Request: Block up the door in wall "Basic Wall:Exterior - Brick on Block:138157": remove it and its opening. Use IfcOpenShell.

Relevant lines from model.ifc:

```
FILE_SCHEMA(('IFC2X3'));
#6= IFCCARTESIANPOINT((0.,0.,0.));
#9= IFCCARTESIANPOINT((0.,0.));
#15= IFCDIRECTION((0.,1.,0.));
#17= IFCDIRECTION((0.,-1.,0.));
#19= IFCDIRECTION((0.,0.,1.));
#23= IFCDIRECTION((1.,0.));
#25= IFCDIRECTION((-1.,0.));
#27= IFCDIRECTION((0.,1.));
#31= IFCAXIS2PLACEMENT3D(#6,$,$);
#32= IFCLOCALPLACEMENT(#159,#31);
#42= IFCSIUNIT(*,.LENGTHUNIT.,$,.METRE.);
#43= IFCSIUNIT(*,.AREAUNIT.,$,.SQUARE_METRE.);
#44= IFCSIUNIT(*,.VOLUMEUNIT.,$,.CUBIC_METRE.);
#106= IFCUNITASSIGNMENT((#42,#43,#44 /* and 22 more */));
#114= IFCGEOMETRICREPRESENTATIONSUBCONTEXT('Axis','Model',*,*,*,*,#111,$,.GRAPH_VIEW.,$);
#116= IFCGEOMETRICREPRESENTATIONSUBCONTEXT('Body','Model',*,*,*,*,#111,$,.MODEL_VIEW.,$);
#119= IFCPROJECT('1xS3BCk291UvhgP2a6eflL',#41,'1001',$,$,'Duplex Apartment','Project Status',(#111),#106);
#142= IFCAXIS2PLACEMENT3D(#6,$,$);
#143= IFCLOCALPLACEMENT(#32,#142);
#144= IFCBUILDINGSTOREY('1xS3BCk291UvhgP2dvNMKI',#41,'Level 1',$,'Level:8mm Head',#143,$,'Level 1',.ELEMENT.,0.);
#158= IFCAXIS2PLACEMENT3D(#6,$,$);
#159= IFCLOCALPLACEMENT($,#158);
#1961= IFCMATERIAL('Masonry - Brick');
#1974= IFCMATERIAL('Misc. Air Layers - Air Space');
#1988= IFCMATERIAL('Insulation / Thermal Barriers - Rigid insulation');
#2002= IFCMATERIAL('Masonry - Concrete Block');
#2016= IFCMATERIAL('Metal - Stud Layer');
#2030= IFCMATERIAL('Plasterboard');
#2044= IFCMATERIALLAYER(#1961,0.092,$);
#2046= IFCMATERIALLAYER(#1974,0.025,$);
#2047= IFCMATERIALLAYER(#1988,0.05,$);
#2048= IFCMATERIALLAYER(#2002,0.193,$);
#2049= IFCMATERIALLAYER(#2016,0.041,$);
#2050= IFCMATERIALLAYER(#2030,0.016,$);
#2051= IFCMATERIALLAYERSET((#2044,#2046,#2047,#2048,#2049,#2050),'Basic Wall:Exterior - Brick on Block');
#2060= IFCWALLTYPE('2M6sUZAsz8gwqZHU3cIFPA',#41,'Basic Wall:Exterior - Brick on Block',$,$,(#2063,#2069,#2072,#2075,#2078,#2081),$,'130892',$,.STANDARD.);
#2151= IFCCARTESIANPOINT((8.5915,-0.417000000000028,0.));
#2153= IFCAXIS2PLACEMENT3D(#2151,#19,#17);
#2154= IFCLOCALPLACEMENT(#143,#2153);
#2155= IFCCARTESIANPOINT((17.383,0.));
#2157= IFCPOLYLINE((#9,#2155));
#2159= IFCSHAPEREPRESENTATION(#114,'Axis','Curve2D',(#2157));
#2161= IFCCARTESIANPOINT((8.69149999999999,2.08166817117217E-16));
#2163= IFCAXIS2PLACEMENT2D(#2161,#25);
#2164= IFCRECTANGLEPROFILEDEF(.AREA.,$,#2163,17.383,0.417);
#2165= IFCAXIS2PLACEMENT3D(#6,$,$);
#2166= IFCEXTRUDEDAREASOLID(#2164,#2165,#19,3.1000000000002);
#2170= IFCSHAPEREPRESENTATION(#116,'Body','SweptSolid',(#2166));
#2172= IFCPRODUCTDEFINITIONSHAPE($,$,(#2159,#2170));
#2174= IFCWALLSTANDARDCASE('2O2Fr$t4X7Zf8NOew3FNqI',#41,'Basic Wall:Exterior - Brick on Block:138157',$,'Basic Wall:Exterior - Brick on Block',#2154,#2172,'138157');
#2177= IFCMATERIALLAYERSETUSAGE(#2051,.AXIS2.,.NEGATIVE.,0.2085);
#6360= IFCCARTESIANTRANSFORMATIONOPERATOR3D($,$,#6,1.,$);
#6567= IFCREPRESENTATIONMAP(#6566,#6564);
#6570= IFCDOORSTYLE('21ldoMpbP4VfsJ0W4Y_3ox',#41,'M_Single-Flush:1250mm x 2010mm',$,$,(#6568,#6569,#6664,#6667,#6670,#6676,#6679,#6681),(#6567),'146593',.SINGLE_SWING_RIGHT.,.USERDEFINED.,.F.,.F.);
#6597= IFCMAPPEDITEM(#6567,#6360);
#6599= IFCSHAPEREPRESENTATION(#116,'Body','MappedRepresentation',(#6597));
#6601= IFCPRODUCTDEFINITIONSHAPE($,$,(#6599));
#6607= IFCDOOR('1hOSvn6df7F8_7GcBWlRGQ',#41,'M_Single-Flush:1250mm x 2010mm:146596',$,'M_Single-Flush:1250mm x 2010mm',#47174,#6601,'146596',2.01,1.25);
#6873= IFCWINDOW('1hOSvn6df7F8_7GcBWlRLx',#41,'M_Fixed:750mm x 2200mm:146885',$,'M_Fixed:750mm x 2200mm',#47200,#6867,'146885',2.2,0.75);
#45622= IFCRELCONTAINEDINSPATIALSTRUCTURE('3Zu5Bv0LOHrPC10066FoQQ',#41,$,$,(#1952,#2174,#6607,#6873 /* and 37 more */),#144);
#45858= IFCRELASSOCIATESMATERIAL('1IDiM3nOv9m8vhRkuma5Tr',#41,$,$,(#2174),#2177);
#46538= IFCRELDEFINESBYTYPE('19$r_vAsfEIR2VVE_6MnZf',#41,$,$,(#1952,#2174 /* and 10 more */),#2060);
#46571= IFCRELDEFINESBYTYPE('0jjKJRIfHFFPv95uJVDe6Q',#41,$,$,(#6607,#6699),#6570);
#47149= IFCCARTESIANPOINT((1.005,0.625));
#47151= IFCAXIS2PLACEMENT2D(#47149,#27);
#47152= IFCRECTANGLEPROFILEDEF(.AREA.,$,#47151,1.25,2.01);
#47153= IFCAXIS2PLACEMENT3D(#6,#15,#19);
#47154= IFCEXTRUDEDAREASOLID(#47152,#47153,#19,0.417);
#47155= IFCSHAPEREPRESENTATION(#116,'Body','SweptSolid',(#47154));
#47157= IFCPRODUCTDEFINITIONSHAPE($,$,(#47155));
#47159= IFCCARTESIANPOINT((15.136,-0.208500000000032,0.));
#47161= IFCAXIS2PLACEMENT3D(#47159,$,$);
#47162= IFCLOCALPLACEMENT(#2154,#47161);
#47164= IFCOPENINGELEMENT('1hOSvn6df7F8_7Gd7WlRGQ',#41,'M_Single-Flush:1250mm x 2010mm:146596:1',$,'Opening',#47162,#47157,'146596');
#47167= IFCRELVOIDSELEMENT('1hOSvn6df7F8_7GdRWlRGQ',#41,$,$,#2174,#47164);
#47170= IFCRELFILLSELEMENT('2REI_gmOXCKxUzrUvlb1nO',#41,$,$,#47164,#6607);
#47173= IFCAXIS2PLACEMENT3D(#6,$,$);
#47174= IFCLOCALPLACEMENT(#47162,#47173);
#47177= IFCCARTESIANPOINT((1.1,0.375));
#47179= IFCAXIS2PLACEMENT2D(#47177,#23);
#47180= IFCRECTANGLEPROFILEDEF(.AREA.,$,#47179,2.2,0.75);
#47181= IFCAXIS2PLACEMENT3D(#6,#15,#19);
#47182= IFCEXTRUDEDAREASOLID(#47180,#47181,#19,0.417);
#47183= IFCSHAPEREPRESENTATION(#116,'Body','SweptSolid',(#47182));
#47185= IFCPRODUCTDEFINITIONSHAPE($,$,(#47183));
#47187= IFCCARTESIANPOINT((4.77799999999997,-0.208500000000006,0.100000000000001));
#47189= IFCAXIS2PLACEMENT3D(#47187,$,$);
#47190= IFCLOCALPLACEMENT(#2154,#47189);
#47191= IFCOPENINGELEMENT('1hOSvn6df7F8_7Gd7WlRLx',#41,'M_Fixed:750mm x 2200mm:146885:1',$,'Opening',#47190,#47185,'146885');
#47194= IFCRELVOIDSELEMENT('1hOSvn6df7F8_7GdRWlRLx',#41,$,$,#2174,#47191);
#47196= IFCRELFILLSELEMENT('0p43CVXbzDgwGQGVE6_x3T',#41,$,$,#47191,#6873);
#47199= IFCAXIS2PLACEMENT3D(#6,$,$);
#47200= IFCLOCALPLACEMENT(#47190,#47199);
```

```python
import ifcopenshell
import ifcopenshell.api.feature
import ifcopenshell.api.root
import ifcopenshell.geom
import ifcopenshell.util.shape

model = ifcopenshell.open("model.ifc")
settings = ifcopenshell.geom.settings()


def volume(element):
    """Net volume in cubic metres, openings subtracted."""
    shape = ifcopenshell.geom.create_shape(settings, element)
    return ifcopenshell.util.shape.get_volume(shape.geometry)


door = model.by_id(6607)
opening = door.FillsVoids[0].RelatingOpeningElement
wall = opening.VoidsElements[0].RelatingBuildingElement
before = volume(wall)

ifcopenshell.api.root.remove_product(model, product=door)
ifcopenshell.api.feature.remove_feature(model, feature=opening)

after = volume(wall)

print(f"wall volume {before:.3f} -> {after:.3f} m3")

model.write("model_rev.ifc")
```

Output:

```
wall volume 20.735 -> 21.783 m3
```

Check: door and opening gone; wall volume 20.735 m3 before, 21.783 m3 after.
